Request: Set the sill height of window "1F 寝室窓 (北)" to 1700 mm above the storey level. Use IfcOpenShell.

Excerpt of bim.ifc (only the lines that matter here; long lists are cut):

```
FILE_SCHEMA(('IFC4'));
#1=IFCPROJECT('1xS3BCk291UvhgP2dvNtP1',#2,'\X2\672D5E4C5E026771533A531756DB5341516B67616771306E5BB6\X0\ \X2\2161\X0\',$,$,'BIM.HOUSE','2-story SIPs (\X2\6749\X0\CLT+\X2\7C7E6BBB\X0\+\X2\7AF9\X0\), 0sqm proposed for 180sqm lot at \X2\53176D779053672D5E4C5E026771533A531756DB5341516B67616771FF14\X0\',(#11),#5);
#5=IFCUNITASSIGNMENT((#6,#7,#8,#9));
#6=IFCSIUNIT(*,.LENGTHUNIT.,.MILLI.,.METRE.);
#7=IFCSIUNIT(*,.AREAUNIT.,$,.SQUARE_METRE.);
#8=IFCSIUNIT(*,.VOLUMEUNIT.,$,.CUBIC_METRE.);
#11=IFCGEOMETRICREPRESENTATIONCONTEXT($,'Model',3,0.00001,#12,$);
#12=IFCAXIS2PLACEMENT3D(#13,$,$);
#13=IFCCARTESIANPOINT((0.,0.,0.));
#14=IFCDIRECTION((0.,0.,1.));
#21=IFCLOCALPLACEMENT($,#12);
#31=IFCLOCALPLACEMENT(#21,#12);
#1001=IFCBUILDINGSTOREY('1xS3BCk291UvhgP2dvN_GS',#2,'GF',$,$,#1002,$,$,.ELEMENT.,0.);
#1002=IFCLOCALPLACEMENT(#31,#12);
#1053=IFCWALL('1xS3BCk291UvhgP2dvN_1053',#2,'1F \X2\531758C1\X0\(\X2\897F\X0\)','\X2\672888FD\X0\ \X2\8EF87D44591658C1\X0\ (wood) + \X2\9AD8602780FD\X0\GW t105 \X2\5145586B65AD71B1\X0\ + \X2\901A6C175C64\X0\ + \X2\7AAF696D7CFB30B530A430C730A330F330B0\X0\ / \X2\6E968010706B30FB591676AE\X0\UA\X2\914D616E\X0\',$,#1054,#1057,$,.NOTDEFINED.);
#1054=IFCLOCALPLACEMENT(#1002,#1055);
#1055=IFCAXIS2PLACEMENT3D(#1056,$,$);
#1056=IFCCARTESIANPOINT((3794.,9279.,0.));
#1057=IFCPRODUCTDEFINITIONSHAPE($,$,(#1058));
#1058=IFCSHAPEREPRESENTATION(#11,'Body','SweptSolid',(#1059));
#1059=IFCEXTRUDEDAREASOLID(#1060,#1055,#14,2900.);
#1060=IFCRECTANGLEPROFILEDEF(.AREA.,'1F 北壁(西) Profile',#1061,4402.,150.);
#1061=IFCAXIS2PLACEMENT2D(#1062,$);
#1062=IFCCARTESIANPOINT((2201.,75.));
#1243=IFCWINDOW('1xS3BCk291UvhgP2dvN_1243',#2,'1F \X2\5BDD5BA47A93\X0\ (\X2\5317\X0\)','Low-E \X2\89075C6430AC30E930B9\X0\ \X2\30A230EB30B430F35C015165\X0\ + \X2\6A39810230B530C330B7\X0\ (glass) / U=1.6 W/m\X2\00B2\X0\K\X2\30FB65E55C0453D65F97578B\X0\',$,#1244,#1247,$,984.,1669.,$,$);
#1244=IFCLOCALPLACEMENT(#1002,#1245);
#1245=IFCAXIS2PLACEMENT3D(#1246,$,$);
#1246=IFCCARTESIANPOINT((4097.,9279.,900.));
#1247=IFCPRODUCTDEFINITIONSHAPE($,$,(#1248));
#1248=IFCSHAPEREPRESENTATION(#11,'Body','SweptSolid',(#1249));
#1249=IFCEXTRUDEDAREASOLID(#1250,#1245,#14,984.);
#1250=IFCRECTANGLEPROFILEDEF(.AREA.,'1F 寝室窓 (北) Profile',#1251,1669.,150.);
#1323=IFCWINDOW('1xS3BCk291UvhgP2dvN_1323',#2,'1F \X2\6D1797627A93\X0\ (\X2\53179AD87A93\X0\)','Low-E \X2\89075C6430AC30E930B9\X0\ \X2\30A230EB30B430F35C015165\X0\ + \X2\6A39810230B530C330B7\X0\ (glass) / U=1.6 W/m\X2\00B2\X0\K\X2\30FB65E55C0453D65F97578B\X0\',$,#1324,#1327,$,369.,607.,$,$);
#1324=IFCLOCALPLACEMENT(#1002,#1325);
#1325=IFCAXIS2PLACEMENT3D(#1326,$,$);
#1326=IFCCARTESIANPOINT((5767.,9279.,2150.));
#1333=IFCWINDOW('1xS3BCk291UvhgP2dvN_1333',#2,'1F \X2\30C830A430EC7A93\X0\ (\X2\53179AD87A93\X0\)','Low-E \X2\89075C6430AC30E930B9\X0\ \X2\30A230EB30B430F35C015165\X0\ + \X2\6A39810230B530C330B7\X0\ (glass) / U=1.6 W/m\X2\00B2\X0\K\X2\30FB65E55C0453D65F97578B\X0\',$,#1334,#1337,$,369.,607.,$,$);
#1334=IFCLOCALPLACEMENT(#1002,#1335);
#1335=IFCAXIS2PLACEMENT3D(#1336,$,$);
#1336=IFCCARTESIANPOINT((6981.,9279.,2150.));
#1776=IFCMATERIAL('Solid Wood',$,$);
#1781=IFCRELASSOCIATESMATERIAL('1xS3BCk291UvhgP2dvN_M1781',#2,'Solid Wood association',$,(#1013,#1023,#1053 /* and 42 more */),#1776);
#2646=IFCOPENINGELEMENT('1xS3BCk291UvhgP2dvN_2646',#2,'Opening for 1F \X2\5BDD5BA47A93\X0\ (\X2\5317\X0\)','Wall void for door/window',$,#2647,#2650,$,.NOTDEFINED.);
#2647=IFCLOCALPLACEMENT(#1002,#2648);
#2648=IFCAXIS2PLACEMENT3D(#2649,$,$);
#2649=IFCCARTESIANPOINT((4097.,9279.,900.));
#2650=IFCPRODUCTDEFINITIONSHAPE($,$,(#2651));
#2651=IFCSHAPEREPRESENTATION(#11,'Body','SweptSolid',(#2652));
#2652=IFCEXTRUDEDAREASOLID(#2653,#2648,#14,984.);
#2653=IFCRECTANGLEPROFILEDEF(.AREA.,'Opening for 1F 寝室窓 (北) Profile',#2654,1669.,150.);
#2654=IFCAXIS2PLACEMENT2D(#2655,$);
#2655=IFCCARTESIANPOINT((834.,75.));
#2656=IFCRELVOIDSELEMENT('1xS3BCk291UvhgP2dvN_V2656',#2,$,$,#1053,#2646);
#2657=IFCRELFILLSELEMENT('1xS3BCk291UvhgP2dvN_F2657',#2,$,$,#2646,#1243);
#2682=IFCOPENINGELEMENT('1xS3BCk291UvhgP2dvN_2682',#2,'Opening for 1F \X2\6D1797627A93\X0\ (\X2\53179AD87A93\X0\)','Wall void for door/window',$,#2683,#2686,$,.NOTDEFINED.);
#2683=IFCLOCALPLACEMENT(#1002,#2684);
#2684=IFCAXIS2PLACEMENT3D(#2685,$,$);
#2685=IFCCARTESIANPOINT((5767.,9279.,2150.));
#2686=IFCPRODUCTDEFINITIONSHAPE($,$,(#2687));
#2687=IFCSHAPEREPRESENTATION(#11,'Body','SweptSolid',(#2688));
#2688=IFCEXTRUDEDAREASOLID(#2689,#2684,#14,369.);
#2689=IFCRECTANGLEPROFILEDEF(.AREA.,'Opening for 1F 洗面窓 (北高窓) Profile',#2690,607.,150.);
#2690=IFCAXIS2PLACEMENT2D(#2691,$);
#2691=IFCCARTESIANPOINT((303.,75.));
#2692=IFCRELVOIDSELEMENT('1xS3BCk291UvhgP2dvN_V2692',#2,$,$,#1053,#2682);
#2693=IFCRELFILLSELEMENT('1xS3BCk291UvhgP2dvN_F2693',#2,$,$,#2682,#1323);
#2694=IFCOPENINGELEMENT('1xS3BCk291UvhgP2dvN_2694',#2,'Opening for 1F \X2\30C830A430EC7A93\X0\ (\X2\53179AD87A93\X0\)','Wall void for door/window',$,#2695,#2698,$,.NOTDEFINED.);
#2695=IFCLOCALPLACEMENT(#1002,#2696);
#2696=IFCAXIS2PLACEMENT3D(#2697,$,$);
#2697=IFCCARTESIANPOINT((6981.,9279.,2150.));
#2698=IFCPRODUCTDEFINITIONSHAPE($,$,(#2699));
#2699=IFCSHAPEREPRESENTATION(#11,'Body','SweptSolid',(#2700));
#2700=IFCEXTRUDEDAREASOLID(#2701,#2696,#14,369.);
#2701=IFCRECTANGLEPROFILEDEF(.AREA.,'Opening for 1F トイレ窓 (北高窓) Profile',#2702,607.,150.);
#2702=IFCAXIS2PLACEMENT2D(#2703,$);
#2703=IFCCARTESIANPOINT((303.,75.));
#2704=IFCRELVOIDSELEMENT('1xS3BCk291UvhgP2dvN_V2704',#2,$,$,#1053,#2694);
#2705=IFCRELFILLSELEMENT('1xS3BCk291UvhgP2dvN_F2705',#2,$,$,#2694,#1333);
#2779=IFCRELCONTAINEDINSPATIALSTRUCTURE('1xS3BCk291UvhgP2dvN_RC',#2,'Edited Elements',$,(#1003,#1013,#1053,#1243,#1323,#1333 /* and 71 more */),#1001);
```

```python
import numpy as np
import ifcopenshell
import ifcopenshell.api.geometry
import ifcopenshell.geom
import ifcopenshell.util.element
import ifcopenshell.util.placement
import ifcopenshell.util.shape
import ifcopenshell.util.unit

model = ifcopenshell.open("bim.ifc")
unit_scale = ifcopenshell.util.unit.calculate_unit_scale(model)

window = model.by_id(1243)
opening = window.FillsVoids[0].RelatingOpeningElement
storey = ifcopenshell.util.element.get_container(window, ifc_class="IfcBuildingStorey")
level = ifcopenshell.util.placement.get_local_placement(storey.ObjectPlacement)[2, 3]

# The opening's origin need not be at the sill, so measure its lowest point.
shape = ifcopenshell.geom.create_shape(ifcopenshell.geom.settings(), opening)
bottom = ifcopenshell.util.shape.get_shape_bottom_elevation(shape, shape.geometry) / unit_scale
dz = level + 1.7 / unit_scale - bottom

shift = np.array([0.0, 0.0, dz])
# The window is not placed relative to its opening, so move both.
for product in (opening, window):
    matrix = ifcopenshell.util.placement.get_local_placement(product.ObjectPlacement)
    matrix[:3, 3] += shift
    ifcopenshell.api.geometry.edit_object_placement(model, product=product, matrix=matrix, is_si=False)

print(f"moved by {dz * unit_scale:+.3f} m")

model.write("bim-out.ifc")
```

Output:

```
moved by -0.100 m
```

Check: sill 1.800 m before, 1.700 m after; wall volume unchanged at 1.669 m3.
